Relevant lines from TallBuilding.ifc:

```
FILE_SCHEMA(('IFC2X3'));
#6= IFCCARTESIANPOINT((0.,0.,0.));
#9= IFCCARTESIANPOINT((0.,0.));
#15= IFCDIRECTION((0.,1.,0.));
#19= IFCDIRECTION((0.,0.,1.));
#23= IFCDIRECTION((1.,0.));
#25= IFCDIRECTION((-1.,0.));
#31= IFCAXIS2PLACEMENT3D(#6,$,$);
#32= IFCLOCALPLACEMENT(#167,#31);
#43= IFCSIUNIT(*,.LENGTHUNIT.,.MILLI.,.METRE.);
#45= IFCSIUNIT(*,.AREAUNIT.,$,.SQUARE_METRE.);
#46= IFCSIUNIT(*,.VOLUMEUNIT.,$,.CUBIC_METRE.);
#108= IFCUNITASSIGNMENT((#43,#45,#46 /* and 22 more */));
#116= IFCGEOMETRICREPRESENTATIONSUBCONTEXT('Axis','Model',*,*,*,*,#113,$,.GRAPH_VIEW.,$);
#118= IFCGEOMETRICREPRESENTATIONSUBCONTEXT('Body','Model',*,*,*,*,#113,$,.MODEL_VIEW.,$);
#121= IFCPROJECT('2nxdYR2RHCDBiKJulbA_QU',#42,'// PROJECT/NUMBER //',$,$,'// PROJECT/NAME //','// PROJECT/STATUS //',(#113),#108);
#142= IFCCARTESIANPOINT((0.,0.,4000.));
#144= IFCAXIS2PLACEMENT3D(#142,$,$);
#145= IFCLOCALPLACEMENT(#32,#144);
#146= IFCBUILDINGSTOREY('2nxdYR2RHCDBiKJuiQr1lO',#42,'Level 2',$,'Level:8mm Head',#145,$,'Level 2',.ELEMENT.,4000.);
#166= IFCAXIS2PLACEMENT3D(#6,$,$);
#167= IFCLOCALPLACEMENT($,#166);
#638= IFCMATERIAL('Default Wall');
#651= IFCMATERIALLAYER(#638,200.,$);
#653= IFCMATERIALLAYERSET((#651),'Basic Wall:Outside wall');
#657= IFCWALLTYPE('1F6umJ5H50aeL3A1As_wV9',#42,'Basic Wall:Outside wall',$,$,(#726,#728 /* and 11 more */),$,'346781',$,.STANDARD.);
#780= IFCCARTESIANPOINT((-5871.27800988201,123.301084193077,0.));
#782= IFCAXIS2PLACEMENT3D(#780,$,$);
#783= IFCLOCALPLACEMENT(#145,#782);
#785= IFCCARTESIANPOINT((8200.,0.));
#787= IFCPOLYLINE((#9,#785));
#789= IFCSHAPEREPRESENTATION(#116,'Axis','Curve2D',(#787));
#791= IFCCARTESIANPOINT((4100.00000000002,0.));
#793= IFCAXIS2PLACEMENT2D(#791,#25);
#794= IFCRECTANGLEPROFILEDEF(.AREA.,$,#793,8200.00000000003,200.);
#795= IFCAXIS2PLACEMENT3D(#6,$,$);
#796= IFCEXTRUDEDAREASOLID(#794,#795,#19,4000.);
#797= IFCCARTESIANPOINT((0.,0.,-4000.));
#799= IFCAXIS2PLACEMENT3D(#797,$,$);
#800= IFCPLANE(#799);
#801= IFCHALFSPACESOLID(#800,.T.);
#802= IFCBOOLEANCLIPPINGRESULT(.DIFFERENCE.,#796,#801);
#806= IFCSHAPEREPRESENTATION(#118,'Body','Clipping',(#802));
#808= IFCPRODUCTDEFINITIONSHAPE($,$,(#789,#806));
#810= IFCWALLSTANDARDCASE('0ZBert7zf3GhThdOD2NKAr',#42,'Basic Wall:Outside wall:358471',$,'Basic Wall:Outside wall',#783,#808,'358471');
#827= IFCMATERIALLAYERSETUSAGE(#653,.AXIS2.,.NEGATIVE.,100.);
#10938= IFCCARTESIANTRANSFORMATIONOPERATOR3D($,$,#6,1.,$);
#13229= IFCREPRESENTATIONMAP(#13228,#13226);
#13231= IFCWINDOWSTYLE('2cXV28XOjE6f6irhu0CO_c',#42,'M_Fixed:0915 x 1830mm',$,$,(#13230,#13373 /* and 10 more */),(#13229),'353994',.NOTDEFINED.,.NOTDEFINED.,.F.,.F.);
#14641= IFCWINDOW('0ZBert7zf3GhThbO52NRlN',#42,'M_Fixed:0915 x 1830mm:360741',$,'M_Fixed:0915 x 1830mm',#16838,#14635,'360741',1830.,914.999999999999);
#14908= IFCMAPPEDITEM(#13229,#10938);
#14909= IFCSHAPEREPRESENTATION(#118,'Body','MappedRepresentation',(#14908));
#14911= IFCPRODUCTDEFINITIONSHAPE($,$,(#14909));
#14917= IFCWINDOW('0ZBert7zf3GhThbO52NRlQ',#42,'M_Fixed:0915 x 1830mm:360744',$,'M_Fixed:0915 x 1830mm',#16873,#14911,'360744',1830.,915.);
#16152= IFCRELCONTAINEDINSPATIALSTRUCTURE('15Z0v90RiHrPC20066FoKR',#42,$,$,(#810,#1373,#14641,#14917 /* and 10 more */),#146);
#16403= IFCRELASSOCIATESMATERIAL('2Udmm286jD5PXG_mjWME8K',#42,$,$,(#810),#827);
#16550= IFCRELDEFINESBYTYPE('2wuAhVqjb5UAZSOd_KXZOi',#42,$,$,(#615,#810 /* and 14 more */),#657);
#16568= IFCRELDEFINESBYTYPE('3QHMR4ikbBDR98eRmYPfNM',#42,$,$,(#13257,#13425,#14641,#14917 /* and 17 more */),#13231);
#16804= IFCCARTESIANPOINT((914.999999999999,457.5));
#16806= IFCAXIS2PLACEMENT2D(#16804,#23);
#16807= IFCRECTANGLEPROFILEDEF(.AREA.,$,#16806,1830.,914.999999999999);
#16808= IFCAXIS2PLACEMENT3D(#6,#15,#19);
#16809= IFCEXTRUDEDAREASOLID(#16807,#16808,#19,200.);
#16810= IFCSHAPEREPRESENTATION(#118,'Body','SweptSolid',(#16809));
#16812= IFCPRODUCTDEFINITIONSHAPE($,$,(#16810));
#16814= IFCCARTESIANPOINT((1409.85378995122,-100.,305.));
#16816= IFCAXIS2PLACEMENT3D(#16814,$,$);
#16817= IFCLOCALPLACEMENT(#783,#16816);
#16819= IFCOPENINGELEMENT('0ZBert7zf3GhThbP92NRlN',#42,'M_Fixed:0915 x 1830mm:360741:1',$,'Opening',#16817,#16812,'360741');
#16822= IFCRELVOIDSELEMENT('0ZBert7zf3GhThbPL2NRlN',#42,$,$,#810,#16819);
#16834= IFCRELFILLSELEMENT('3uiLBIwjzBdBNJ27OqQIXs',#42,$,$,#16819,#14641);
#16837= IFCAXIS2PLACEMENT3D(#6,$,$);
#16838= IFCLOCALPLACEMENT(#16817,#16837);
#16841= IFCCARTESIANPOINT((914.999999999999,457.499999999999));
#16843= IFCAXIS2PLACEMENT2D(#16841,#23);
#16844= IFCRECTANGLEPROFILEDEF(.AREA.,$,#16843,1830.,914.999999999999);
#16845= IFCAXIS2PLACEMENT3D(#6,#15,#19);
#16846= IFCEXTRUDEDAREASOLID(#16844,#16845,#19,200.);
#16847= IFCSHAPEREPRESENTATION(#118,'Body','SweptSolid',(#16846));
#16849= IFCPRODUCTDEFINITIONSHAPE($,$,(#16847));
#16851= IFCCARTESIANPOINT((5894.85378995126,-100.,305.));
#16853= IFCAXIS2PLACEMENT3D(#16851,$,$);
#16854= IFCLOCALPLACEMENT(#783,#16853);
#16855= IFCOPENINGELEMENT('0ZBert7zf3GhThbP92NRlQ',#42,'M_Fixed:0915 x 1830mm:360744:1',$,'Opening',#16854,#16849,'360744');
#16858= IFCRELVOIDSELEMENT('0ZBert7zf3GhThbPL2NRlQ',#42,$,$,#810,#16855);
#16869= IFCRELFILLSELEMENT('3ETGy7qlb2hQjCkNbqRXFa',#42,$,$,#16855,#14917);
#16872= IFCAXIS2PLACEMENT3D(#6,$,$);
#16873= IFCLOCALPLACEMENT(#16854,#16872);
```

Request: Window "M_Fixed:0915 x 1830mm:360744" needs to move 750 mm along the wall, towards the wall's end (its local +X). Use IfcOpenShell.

```python
import ifcopenshell
import ifcopenshell.api.geometry
import ifcopenshell.util.placement
import ifcopenshell.util.unit

model = ifcopenshell.open("TallBuilding.ifc")
unit_scale = ifcopenshell.util.unit.calculate_unit_scale(model)

window = model.by_guid("0ZBert7zf3GhThbO52NRlQ")
opening = window.FillsVoids[0].RelatingOpeningElement
wall = opening.VoidsElements[0].RelatingBuildingElement

wall_matrix = ifcopenshell.util.placement.get_local_placement(wall.ObjectPlacement)
shift = wall_matrix[:3, 0] * 0.75 / unit_scale
before = ifcopenshell.util.placement.get_local_placement(window.ObjectPlacement)[:3, 3].copy()

# The window is placed relative to its opening, so it follows when the opening moves.
matrix = ifcopenshell.util.placement.get_local_placement(opening.ObjectPlacement)
matrix[:3, 3] += shift
ifcopenshell.api.geometry.edit_object_placement(
    model, product=opening, matrix=matrix, is_si=False, should_transform_children=True
)

after = ifcopenshell.util.placement.get_local_placement(window.ObjectPlacement)[:3, 3]
print("window moved by", (after - before).round(3) + 0.0)

model.write("TallBuilding_rev.ifc")
```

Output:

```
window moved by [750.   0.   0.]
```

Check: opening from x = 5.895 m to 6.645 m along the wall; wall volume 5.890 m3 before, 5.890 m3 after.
